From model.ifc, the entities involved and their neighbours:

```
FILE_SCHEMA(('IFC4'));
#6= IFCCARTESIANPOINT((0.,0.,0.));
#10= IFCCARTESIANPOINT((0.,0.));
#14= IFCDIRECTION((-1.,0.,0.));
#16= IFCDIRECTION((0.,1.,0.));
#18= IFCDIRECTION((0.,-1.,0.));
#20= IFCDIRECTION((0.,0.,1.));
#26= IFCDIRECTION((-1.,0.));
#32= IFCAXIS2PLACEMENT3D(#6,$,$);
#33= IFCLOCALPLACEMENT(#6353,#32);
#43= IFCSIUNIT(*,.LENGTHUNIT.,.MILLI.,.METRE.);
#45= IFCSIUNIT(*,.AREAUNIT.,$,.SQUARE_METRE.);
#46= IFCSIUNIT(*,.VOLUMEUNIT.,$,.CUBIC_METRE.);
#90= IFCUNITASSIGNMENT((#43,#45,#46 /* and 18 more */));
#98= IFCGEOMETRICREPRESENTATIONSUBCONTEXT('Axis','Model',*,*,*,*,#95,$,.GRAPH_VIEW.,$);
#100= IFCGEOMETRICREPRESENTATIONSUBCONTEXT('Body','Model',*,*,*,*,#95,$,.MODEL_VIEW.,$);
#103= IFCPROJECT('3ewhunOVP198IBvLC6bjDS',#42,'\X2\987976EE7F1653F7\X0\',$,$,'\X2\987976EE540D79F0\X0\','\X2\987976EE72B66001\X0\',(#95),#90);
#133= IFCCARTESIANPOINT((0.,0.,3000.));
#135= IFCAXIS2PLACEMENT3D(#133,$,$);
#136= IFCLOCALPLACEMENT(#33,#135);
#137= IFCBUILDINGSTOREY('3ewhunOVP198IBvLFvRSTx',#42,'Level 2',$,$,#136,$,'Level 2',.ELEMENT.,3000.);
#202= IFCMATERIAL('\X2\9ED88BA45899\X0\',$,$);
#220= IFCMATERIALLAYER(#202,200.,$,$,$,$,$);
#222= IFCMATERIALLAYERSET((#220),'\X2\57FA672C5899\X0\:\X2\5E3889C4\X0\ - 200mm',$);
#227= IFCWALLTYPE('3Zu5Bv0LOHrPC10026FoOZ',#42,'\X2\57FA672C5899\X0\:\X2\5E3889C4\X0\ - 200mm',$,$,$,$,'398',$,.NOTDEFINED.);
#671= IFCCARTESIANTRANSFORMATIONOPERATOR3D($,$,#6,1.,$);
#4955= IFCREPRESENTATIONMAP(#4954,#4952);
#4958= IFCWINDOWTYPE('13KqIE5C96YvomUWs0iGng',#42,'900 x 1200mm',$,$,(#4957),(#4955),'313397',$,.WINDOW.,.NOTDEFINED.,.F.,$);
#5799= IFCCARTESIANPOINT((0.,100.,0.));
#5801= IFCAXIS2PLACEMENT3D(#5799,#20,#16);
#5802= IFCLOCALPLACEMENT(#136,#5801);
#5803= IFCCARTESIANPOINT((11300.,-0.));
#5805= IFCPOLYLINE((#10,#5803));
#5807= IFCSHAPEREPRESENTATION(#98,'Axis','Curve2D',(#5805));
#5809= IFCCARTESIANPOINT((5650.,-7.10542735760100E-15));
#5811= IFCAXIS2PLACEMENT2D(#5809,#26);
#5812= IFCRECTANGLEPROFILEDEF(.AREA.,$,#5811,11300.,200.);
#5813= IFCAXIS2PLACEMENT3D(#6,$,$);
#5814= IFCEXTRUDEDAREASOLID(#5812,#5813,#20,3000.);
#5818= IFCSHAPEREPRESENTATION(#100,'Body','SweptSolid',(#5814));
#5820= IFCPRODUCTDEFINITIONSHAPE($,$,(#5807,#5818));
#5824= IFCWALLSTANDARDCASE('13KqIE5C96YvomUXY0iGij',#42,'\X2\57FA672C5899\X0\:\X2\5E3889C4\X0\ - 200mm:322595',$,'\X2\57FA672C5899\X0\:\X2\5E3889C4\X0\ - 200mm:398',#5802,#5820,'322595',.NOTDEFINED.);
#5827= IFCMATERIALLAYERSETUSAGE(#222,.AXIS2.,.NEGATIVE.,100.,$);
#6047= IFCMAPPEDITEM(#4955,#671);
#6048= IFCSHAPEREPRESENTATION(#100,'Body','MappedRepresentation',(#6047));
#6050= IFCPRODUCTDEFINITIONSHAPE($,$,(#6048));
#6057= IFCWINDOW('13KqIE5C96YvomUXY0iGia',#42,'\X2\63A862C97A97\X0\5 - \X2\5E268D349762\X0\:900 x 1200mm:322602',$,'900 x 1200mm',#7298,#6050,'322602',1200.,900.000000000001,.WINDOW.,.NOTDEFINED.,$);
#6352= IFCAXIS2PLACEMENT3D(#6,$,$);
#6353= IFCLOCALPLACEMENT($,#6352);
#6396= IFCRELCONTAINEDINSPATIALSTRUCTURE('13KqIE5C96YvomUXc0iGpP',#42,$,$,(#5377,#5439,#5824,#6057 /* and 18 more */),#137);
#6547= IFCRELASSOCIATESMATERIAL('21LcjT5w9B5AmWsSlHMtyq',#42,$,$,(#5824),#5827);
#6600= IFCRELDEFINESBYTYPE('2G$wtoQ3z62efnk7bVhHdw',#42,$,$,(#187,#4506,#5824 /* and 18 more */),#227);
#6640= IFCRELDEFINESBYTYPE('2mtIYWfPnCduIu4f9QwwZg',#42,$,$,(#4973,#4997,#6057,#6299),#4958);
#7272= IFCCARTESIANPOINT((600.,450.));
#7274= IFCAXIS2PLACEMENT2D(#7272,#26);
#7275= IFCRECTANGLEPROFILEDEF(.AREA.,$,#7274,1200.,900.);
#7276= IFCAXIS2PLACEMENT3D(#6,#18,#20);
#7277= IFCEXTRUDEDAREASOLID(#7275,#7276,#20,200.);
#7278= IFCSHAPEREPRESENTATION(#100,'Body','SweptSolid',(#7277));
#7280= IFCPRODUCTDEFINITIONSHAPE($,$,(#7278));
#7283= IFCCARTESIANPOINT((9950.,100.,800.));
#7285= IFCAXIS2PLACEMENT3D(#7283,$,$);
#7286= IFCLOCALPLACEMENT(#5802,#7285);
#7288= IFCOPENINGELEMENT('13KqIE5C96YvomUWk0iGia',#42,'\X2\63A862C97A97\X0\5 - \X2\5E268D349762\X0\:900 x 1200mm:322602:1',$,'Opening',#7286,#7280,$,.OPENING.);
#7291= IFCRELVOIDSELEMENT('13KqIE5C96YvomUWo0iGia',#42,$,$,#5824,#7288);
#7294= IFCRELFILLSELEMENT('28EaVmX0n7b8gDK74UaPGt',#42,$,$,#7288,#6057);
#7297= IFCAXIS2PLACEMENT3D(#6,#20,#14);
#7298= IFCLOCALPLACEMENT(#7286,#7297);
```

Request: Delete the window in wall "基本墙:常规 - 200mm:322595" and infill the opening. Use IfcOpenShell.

```python
import ifcopenshell
import ifcopenshell.api.feature
import ifcopenshell.api.root
import ifcopenshell.geom
import ifcopenshell.util.shape

model = ifcopenshell.open("model.ifc")
settings = ifcopenshell.geom.settings()


def volume(element):
    """Net volume in cubic metres, openings subtracted."""
    shape = ifcopenshell.geom.create_shape(settings, element)
    return ifcopenshell.util.shape.get_volume(shape.geometry)


window = model.by_guid("13KqIE5C96YvomUXY0iGia")
opening = window.FillsVoids[0].RelatingOpeningElement
wall = opening.VoidsElements[0].RelatingBuildingElement
before = volume(wall)

ifcopenshell.api.root.remove_product(model, product=window)
ifcopenshell.api.feature.remove_feature(model, feature=opening)

after = volume(wall)

print(f"wall volume {before:.3f} -> {after:.3f} m3")

model.write("model-out.ifc")
```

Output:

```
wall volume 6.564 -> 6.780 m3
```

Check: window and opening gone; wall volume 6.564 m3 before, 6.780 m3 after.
